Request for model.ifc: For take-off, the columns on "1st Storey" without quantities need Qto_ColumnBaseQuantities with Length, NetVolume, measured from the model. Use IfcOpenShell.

First a look at what the model holds.

```python
import ifcopenshell
import ifcopenshell.util.element
import ifcopenshell.util.unit

model = ifcopenshell.open("model.ifc")
print(model.schema)
for unit_type in ("LENGTHUNIT", "AREAUNIT", "VOLUMEUNIT"):
    print(unit_type, ifcopenshell.util.unit.calculate_unit_scale(model, unit_type))
storey = next(s for s in model.by_type("IfcBuildingStorey") if s.Name == "1st Storey")
columns = [e for e in ifcopenshell.util.element.get_decomposition(storey) if e.is_a("IfcColumn")]
for e in sorted(columns, key=lambda e: e.id()):
    print(e.id(), e.is_a(), e.Name, list(ifcopenshell.util.element.get_psets(e, qtos_only=True)), sep=" | ")
```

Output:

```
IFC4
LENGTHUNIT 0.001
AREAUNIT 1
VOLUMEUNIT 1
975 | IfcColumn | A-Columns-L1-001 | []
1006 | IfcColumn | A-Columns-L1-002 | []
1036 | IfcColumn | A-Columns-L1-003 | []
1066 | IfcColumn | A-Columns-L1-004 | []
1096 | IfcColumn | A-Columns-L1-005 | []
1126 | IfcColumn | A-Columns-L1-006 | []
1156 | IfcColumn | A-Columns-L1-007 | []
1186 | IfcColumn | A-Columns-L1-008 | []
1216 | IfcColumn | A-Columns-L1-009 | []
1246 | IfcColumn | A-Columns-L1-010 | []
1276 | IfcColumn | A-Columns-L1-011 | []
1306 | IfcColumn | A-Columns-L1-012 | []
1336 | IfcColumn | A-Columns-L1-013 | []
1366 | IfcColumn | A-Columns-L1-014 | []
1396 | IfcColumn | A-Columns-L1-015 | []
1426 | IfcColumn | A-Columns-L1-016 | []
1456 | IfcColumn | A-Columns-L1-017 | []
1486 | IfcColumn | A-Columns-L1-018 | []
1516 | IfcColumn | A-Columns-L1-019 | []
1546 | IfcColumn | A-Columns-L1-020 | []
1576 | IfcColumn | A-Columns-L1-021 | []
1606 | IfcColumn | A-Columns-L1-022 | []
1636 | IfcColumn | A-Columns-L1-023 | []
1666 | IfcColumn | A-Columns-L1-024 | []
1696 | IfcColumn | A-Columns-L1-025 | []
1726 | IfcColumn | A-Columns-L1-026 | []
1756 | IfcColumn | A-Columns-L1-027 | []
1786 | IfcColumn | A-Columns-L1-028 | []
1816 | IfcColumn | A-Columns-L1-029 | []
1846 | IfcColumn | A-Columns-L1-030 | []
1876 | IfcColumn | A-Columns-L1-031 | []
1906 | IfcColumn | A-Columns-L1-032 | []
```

```python
import ifcopenshell
import ifcopenshell.api.pset
import ifcopenshell.geom
import ifcopenshell.util.element
import ifcopenshell.util.shape
import ifcopenshell.util.unit

model = ifcopenshell.open("model.ifc")
unit_scale = ifcopenshell.util.unit.calculate_unit_scale(model)
volume_scale = ifcopenshell.util.unit.calculate_unit_scale(model, "VOLUMEUNIT")
settings = ifcopenshell.geom.settings()

storey = next(s for s in model.by_type("IfcBuildingStorey") if s.Name == "1st Storey")
columns = [e for e in ifcopenshell.util.element.get_decomposition(storey) if e.is_a("IfcColumn")]

for e in sorted(columns, key=lambda e: e.id()):
    if ifcopenshell.util.element.get_psets(e, qtos_only=True, should_inherit=False):
        continue
    # Geometry comes back in metres, in the element's own axes.
    shape = ifcopenshell.geom.create_shape(settings, e)
    values = {
        "Length": ifcopenshell.util.shape.get_z(shape.geometry) / unit_scale,
        "NetVolume": ifcopenshell.util.shape.get_volume(shape.geometry) / volume_scale,
    }
    qto = ifcopenshell.api.pset.add_qto(model, product=e, name="Qto_ColumnBaseQuantities")
    ifcopenshell.api.pset.edit_qto(model, qto=qto, properties=values)
    print(e.id(), {k: round(v, 3) for k, v in values.items()})

model.write("model_v2.ifc")
```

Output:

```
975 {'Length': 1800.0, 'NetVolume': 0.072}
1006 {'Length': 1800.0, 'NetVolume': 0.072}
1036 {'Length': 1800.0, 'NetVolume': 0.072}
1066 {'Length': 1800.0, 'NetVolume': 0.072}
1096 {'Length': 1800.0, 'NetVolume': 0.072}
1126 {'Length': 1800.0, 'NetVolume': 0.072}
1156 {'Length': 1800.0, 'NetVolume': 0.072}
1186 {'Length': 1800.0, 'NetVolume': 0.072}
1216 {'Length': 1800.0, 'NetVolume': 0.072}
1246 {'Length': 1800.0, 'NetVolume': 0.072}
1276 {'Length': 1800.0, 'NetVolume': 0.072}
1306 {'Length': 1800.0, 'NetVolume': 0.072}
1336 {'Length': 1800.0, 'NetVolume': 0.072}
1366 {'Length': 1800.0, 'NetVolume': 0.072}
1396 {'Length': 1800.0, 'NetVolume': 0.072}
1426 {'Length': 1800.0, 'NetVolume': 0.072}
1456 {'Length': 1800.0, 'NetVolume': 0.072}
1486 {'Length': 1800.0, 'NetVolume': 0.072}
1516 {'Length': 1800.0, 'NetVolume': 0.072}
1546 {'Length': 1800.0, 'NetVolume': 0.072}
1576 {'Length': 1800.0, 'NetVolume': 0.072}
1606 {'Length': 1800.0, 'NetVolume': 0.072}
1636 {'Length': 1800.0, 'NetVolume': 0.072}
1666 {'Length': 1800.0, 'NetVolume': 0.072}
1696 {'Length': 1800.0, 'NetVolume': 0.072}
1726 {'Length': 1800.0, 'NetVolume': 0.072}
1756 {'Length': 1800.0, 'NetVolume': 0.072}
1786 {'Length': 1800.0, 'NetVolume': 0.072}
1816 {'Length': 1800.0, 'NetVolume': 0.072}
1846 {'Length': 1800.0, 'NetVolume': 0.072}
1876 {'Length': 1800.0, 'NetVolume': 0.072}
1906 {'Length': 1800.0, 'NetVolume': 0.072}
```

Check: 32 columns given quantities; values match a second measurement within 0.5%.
